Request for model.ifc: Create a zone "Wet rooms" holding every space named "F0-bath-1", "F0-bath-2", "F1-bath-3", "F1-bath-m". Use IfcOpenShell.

First a look at what the model holds.

```python
import ifcopenshell

model = ifcopenshell.open("model.ifc")
print(model.schema)
seen = {}
for space in model.by_type("IfcSpace"):
    seen[space.LongName] = seen.get(space.LongName, 0) + 1
for name, count in sorted(seen.items(), key=str):
    print(count, "x", name)
print("zones:", [z.Name for z in model.by_type("IfcZone")][:20])
```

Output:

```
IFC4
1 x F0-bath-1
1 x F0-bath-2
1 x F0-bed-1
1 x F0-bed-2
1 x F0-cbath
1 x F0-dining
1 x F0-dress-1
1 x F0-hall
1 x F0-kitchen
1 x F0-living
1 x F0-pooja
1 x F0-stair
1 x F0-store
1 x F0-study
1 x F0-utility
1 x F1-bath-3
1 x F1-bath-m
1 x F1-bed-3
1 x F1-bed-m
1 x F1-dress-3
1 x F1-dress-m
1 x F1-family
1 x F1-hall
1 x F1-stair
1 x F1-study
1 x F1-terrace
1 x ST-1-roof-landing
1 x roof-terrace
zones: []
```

```python
import ifcopenshell
import ifcopenshell.api.group
import ifcopenshell.api.root

model = ifcopenshell.open("model.ifc")

names = {"F0-bath-1", "F0-bath-2", "F1-bath-3", "F1-bath-m"}
spaces = [s for s in model.by_type("IfcSpace") if s.LongName in names]

zone = ifcopenshell.api.root.create_entity(model, ifc_class="IfcZone", name="Wet rooms")
ifcopenshell.api.group.assign_group(model, products=spaces, group=zone)
print(len(spaces), "spaces in", zone.Name)

model.write("model_edited.ifc")
```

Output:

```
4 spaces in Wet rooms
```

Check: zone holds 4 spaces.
